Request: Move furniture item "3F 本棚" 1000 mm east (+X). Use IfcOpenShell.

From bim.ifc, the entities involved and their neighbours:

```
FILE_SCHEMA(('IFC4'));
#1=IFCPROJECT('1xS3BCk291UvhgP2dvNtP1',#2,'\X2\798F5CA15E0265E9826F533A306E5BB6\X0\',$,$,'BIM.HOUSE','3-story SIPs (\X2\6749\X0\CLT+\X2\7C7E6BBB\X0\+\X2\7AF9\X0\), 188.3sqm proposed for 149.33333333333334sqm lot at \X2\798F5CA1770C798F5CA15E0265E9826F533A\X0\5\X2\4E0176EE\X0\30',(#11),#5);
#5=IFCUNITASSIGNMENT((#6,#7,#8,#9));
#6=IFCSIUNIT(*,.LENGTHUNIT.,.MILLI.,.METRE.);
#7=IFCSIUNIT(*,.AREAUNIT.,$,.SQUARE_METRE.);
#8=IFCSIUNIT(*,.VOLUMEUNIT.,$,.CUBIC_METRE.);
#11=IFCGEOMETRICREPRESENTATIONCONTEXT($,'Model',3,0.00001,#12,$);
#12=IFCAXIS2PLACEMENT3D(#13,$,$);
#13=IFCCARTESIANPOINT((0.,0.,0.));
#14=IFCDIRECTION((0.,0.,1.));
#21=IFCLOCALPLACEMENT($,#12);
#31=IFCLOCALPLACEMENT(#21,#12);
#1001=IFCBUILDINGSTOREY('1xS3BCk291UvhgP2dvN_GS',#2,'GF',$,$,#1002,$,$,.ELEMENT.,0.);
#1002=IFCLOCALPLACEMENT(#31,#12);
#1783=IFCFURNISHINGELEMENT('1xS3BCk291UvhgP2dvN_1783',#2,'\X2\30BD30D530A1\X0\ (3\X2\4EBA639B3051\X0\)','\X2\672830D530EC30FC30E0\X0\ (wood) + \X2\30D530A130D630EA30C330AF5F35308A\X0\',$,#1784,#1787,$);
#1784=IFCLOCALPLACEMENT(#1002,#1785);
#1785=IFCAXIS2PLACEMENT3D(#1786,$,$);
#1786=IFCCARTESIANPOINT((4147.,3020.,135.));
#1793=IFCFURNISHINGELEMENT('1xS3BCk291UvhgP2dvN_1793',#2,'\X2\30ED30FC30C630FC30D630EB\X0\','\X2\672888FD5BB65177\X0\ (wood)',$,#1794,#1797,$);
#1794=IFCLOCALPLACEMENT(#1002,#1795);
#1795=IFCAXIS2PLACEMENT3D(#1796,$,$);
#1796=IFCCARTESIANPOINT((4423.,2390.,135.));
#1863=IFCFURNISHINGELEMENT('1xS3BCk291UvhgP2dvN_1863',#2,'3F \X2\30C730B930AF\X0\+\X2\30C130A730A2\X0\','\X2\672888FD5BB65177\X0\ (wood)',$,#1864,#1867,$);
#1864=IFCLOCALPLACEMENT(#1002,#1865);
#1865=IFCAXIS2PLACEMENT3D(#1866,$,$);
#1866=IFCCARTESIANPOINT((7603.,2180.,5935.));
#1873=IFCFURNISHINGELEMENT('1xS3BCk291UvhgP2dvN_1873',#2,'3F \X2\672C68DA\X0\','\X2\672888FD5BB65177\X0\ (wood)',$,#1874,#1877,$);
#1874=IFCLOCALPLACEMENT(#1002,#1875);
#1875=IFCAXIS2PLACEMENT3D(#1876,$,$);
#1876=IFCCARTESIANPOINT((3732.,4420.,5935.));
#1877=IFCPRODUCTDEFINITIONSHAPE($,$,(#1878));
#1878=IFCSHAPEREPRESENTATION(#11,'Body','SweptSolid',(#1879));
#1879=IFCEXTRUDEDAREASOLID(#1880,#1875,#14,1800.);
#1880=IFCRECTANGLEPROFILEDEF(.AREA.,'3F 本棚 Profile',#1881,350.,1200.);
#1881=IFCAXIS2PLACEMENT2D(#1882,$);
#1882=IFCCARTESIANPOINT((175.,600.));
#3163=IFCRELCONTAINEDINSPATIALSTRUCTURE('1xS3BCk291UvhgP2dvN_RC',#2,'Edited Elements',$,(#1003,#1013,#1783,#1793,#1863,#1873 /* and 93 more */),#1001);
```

```python
import ifcopenshell
import ifcopenshell.api.geometry
import ifcopenshell.util.placement
import ifcopenshell.util.unit

model = ifcopenshell.open("bim.ifc")
unit_scale = ifcopenshell.util.unit.calculate_unit_scale(model)

item = model.by_guid("1xS3BCk291UvhgP2dvN_1873")
matrix = ifcopenshell.util.placement.get_local_placement(item.ObjectPlacement)
matrix[0, 3] += 1 / unit_scale
ifcopenshell.api.geometry.edit_object_placement(model, product=item, matrix=matrix, is_si=False)

print(ifcopenshell.util.placement.get_local_placement(item.ObjectPlacement).round(3) + 0.0)

model.write("bim_v2.ifc")
```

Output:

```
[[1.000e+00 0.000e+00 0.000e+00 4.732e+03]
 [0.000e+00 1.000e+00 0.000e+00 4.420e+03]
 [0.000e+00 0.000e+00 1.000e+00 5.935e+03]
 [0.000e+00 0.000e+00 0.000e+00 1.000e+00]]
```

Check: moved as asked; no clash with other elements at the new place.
